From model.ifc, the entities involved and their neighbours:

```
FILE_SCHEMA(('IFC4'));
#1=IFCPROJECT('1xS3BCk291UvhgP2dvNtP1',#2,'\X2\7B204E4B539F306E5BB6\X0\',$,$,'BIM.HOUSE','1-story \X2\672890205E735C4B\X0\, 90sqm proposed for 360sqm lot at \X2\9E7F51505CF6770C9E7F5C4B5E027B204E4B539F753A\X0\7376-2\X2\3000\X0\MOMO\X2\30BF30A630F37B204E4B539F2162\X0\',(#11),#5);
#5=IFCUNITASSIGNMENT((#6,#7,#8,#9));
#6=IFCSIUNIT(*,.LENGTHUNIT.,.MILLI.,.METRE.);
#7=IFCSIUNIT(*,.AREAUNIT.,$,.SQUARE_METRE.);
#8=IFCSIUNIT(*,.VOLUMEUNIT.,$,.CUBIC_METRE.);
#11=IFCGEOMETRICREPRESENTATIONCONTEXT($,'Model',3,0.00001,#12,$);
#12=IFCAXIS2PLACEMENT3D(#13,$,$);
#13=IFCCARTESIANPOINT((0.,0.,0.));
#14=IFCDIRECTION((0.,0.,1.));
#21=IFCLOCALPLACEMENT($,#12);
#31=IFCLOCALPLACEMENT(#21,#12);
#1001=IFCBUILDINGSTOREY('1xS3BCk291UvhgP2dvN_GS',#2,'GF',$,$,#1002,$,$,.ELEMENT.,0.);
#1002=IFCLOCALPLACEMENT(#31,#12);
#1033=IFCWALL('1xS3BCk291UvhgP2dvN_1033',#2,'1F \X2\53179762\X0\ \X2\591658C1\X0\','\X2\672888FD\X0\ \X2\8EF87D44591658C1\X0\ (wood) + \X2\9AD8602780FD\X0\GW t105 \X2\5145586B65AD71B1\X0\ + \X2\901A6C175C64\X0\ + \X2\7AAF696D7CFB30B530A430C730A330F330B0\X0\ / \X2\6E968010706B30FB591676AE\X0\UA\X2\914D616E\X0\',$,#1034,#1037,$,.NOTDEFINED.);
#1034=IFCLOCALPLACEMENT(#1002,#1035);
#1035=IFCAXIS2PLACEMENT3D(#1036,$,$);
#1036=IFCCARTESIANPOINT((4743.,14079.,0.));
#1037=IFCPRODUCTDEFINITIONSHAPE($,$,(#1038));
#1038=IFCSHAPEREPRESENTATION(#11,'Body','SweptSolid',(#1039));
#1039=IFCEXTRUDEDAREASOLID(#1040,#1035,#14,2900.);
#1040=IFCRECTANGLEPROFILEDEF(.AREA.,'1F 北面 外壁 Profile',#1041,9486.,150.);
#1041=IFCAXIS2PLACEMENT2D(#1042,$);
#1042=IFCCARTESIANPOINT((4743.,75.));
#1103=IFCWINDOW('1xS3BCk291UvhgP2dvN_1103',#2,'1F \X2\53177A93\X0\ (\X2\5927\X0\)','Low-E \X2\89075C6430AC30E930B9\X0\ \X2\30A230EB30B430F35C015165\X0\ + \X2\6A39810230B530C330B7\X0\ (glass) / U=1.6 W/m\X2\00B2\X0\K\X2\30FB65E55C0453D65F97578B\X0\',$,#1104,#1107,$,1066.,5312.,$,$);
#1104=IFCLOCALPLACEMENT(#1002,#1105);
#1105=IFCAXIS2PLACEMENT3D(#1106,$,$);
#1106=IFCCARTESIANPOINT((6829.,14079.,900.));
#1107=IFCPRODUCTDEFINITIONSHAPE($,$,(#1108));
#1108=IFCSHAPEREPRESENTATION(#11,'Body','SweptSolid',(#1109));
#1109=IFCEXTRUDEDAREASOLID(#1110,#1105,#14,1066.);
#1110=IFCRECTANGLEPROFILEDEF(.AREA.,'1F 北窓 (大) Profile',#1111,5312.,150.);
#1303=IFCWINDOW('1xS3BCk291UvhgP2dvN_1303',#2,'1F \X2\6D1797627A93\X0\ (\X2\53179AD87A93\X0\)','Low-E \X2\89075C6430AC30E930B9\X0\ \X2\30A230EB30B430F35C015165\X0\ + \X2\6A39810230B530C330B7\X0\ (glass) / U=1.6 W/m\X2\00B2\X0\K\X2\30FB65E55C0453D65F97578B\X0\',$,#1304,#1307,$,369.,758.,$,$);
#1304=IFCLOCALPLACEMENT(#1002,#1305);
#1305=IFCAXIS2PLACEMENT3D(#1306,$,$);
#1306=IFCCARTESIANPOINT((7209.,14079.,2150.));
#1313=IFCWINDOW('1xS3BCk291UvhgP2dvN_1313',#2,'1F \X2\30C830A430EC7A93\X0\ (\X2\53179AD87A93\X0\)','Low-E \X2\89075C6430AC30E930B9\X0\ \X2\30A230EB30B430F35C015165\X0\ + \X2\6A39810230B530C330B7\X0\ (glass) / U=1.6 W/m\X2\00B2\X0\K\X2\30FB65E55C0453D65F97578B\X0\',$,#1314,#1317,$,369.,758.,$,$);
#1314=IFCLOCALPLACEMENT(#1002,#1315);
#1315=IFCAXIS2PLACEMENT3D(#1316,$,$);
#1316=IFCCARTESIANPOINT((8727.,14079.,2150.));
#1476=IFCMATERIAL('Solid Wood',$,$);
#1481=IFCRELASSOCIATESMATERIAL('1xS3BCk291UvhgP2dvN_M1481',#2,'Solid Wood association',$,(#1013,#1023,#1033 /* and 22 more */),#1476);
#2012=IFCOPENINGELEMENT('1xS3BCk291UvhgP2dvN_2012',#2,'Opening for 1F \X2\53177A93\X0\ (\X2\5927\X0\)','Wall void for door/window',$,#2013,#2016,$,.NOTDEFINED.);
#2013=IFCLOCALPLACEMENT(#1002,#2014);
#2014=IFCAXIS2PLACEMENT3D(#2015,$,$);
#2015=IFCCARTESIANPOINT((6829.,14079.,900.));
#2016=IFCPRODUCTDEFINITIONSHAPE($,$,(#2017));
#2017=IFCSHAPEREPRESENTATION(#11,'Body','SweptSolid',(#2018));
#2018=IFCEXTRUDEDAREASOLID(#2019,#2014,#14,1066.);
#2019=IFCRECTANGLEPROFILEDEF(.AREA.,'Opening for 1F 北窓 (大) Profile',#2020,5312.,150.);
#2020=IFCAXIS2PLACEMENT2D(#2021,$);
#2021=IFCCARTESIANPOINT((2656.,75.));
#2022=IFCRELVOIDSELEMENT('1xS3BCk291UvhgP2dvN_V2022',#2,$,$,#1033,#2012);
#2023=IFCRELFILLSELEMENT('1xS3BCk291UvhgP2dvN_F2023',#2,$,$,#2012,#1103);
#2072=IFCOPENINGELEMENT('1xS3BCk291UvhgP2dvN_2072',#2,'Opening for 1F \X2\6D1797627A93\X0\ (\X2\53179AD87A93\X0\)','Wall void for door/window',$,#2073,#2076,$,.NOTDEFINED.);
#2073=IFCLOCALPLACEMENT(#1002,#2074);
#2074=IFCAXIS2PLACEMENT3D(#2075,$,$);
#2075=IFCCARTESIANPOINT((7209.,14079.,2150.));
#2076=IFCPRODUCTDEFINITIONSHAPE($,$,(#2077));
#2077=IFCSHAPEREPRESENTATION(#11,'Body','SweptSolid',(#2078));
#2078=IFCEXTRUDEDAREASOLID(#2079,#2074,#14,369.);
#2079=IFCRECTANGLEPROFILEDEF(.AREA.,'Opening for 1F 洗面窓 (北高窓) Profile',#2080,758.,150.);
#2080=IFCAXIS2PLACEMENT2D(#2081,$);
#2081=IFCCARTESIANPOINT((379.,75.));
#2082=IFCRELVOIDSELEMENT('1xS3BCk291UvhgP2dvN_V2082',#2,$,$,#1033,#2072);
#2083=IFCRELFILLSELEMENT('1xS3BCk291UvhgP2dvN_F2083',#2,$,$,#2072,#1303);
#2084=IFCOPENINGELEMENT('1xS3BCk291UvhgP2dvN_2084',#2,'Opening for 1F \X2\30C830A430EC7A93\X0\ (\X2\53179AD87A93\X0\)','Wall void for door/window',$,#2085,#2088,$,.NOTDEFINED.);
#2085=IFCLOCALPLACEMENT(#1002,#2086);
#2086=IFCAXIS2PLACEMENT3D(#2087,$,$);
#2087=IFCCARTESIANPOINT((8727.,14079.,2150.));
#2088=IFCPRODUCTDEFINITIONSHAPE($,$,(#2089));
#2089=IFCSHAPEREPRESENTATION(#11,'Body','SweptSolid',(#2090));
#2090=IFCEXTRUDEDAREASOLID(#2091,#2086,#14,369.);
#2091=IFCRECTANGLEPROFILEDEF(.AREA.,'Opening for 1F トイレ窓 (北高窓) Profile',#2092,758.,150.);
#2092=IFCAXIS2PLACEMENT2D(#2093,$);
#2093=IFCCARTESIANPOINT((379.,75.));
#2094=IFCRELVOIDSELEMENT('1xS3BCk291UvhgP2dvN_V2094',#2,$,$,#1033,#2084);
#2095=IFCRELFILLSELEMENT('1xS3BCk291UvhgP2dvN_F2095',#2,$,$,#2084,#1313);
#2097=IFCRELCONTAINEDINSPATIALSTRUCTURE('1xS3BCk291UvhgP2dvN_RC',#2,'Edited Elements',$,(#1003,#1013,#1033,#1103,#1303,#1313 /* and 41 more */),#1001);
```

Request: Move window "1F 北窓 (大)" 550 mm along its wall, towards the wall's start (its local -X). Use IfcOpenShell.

```python
import ifcopenshell
import ifcopenshell.api.geometry
import ifcopenshell.util.placement

model = ifcopenshell.open("model.ifc")

window = model.by_guid("1xS3BCk291UvhgP2dvN_1103")
opening = window.FillsVoids[0].RelatingOpeningElement
wall = opening.VoidsElements[0].RelatingBuildingElement

wall_matrix = ifcopenshell.util.placement.get_local_placement(wall.ObjectPlacement)
shift = wall_matrix[:3, 0] * -550.0
before = ifcopenshell.util.placement.get_local_placement(window.ObjectPlacement)[:3, 3].copy()

# The window is not placed relative to its opening, so move both.
for product in (opening, window):
    matrix = ifcopenshell.util.placement.get_local_placement(product.ObjectPlacement)
    matrix[:3, 3] += shift
    ifcopenshell.api.geometry.edit_object_placement(model, product=product, matrix=matrix, is_si=False)

after = ifcopenshell.util.placement.get_local_placement(window.ObjectPlacement)[:3, 3]
print("window moved by", (after - before).round(3) + 0.0)

model.write("model_edited.ifc")
```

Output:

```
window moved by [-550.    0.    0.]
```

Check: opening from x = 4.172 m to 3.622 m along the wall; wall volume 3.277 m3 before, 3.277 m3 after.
